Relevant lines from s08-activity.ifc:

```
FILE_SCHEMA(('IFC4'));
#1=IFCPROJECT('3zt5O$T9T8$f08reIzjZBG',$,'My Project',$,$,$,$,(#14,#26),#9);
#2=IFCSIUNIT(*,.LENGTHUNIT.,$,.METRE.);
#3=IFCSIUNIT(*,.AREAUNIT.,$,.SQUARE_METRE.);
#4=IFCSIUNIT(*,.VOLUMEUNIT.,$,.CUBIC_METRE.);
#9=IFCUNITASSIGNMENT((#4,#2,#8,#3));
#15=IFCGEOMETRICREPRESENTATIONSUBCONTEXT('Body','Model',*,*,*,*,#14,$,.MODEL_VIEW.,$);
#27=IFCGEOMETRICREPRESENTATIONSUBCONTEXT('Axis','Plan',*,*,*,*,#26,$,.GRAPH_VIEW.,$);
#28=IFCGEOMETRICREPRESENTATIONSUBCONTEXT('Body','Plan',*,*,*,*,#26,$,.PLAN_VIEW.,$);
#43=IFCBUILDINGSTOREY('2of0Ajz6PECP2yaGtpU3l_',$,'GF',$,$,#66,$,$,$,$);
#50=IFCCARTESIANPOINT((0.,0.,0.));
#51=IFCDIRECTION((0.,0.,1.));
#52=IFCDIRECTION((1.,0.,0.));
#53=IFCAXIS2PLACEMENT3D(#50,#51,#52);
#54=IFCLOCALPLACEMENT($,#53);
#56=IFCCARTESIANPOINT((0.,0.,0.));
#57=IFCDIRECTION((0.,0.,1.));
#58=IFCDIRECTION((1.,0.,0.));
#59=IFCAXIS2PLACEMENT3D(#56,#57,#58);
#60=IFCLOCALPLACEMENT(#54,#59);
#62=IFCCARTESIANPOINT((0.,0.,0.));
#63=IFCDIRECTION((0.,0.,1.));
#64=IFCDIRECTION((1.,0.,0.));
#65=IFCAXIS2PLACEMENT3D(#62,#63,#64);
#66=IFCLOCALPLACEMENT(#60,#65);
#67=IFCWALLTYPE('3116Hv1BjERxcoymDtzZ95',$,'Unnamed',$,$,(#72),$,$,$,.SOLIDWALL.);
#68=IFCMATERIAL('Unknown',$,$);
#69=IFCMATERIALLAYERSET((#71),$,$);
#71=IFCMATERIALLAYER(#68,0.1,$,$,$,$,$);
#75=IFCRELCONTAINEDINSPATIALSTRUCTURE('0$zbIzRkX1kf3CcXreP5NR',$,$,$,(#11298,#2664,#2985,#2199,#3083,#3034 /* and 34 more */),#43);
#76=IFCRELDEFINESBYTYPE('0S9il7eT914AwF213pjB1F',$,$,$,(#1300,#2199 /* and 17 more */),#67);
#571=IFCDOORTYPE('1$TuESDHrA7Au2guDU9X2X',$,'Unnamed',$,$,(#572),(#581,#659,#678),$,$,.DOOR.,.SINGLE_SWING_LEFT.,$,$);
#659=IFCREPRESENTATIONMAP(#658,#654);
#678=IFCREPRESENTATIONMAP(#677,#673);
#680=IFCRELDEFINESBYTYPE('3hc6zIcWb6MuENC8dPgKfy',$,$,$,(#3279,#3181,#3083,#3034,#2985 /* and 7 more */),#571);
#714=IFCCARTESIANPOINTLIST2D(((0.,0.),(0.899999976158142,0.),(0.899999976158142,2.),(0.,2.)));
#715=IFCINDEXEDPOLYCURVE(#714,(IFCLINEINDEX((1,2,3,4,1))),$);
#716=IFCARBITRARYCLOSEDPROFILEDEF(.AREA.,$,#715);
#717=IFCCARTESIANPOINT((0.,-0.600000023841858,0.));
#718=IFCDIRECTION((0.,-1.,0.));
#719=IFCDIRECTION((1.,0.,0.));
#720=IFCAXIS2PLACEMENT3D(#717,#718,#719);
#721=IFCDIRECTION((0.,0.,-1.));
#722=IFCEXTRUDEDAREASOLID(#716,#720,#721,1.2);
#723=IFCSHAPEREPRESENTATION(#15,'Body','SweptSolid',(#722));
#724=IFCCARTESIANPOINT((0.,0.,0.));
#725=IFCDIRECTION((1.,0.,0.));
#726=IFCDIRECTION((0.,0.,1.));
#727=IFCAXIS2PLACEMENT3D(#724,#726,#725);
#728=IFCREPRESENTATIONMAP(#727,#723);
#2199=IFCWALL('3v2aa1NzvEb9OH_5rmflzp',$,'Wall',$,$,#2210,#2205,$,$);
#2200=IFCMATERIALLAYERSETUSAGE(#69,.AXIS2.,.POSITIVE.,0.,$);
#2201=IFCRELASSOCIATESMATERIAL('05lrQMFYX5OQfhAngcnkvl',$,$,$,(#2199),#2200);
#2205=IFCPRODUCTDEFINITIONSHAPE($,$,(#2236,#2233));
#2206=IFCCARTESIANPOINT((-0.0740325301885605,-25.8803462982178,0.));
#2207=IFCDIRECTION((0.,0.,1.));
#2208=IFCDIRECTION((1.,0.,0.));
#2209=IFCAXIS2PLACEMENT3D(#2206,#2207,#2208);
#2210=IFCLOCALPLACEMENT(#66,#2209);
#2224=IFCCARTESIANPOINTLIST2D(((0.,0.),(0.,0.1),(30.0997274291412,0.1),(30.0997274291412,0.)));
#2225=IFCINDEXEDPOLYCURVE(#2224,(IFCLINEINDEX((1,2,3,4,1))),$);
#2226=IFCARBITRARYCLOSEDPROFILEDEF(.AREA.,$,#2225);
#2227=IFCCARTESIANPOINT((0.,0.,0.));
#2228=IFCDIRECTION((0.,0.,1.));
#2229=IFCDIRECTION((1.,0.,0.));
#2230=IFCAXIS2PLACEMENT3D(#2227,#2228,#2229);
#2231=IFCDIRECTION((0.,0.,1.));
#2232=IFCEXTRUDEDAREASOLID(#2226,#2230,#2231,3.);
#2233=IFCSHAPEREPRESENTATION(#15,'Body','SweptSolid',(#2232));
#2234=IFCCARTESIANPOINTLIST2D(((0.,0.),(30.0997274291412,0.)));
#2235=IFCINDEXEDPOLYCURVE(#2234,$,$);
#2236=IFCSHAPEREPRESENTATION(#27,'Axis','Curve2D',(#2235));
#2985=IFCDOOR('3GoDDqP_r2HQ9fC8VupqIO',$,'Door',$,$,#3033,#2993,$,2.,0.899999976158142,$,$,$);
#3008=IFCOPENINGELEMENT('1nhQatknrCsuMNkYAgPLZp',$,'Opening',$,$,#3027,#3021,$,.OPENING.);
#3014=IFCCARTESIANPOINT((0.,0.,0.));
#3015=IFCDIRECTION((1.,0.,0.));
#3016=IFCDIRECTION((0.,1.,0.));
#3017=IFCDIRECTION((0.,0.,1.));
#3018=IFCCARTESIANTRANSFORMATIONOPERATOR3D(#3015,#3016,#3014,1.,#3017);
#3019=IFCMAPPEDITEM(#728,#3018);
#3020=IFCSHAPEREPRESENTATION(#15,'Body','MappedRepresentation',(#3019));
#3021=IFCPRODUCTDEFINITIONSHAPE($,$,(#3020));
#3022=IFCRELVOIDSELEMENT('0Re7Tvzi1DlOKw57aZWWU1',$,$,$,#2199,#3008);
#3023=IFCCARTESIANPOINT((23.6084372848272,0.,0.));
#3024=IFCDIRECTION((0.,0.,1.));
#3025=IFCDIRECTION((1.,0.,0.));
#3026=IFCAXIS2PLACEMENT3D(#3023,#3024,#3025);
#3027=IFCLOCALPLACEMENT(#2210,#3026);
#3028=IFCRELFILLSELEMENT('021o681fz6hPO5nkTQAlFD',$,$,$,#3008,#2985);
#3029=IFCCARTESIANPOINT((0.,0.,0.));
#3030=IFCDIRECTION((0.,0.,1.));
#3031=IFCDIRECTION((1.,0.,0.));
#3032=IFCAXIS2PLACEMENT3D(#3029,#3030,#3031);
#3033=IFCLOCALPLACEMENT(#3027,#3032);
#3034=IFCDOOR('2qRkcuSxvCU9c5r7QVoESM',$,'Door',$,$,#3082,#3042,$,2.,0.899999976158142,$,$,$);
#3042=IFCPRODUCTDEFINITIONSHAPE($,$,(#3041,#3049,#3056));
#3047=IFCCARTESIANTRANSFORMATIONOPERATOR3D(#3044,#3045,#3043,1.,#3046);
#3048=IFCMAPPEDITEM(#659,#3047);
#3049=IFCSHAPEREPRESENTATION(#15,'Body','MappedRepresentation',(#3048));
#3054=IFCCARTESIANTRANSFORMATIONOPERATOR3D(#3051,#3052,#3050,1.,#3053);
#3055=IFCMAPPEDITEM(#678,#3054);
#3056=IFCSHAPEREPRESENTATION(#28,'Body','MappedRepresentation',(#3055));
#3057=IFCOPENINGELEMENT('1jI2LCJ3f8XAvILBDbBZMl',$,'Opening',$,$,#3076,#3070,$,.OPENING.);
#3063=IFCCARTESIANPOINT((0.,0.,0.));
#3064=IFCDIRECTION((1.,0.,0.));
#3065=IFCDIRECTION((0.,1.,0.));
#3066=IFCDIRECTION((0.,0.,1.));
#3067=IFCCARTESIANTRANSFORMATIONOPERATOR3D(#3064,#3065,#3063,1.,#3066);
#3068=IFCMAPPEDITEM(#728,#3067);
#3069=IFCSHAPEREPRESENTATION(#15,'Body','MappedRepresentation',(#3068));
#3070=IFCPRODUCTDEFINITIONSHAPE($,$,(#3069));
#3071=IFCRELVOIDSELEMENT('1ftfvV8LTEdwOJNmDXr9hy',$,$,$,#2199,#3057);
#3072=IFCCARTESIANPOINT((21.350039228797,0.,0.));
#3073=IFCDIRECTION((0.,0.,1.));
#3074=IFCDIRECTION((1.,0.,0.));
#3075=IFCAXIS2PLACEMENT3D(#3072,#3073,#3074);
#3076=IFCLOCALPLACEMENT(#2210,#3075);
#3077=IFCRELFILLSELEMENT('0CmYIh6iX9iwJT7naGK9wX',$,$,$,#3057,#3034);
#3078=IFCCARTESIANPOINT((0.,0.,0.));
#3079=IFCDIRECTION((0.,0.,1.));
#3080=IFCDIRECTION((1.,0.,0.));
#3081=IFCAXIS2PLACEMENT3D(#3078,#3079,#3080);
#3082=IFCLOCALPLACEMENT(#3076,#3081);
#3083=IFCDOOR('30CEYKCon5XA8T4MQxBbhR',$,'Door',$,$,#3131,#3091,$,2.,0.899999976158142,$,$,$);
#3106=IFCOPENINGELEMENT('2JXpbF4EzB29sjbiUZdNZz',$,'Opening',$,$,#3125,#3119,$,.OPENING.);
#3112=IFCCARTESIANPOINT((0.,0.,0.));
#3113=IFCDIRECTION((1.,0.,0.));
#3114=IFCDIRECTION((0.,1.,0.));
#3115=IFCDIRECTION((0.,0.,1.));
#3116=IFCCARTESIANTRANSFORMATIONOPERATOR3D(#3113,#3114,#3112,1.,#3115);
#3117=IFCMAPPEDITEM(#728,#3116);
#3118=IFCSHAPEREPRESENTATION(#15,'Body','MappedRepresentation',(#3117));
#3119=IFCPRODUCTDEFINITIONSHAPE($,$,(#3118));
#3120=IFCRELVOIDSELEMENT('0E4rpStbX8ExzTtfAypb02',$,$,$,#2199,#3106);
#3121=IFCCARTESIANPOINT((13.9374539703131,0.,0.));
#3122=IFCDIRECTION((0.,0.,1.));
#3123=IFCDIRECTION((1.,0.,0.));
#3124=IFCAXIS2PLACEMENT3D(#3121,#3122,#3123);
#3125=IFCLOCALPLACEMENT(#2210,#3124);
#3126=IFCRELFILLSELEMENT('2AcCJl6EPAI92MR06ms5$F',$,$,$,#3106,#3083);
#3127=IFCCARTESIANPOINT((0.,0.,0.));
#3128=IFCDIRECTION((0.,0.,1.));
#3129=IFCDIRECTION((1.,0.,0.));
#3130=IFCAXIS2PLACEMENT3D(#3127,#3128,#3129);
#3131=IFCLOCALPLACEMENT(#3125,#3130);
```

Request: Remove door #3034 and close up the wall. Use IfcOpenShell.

```python
import ifcopenshell
import ifcopenshell.api.feature
import ifcopenshell.api.root
import ifcopenshell.geom
import ifcopenshell.util.shape

model = ifcopenshell.open("s08-activity.ifc")
settings = ifcopenshell.geom.settings()


def volume(element):
    """Net volume in cubic metres, openings subtracted."""
    shape = ifcopenshell.geom.create_shape(settings, element)
    return ifcopenshell.util.shape.get_volume(shape.geometry)


door = model.by_guid("2qRkcuSxvCU9c5r7QVoESM")
opening = door.FillsVoids[0].RelatingOpeningElement
wall = opening.VoidsElements[0].RelatingBuildingElement
before = volume(wall)

ifcopenshell.api.root.remove_product(model, product=door)
ifcopenshell.api.feature.remove_feature(model, feature=opening)

after = volume(wall)

print(f"wall volume {before:.3f} -> {after:.3f} m3")

model.write("s08-activity_edited.ifc")
```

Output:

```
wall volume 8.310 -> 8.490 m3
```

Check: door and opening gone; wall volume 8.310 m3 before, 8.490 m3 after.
